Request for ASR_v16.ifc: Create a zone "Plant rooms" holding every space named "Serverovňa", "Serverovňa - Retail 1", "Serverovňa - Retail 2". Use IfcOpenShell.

First a look at what the model holds.

```python
import ifcopenshell

model = ifcopenshell.open("ASR_v16.ifc")
print(model.schema)
seen = {}
for space in model.by_type("IfcSpace"):
    seen[space.LongName] = seen.get(space.LongName, 0) + 1
for name, count in sorted(seen.items(), key=str):
    print(count, "x", name)
print("zones:", [z.Name for z in model.by_type("IfcZone")][:20])
```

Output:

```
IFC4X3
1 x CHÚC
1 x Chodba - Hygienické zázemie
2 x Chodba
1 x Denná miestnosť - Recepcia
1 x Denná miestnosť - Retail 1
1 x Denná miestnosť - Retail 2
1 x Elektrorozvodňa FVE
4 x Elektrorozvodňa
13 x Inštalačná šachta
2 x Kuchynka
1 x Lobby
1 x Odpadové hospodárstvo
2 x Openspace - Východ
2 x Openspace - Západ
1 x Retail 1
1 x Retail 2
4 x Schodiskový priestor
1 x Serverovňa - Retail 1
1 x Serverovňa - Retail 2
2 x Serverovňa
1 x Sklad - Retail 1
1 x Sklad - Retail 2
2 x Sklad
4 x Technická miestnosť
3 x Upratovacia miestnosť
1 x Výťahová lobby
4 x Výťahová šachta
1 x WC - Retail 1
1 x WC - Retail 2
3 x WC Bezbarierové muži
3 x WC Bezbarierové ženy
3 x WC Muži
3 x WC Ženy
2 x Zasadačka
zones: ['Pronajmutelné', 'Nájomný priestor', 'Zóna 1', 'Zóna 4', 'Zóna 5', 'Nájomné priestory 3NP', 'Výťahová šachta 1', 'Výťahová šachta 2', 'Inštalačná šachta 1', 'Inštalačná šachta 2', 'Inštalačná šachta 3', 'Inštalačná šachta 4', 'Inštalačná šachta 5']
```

```python
import ifcopenshell
import ifcopenshell.api.group
import ifcopenshell.api.root

model = ifcopenshell.open("ASR_v16.ifc")

names = {"Serverovňa", "Serverovňa - Retail 1", "Serverovňa - Retail 2"}
spaces = [s for s in model.by_type("IfcSpace") if s.LongName in names]

zone = ifcopenshell.api.root.create_entity(model, ifc_class="IfcZone", name="Plant rooms")
ifcopenshell.api.group.assign_group(model, products=spaces, group=zone)
print(len(spaces), "spaces in", zone.Name)

model.write("ASR_v16_rev.ifc")
```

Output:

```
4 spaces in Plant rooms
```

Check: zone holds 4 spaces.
